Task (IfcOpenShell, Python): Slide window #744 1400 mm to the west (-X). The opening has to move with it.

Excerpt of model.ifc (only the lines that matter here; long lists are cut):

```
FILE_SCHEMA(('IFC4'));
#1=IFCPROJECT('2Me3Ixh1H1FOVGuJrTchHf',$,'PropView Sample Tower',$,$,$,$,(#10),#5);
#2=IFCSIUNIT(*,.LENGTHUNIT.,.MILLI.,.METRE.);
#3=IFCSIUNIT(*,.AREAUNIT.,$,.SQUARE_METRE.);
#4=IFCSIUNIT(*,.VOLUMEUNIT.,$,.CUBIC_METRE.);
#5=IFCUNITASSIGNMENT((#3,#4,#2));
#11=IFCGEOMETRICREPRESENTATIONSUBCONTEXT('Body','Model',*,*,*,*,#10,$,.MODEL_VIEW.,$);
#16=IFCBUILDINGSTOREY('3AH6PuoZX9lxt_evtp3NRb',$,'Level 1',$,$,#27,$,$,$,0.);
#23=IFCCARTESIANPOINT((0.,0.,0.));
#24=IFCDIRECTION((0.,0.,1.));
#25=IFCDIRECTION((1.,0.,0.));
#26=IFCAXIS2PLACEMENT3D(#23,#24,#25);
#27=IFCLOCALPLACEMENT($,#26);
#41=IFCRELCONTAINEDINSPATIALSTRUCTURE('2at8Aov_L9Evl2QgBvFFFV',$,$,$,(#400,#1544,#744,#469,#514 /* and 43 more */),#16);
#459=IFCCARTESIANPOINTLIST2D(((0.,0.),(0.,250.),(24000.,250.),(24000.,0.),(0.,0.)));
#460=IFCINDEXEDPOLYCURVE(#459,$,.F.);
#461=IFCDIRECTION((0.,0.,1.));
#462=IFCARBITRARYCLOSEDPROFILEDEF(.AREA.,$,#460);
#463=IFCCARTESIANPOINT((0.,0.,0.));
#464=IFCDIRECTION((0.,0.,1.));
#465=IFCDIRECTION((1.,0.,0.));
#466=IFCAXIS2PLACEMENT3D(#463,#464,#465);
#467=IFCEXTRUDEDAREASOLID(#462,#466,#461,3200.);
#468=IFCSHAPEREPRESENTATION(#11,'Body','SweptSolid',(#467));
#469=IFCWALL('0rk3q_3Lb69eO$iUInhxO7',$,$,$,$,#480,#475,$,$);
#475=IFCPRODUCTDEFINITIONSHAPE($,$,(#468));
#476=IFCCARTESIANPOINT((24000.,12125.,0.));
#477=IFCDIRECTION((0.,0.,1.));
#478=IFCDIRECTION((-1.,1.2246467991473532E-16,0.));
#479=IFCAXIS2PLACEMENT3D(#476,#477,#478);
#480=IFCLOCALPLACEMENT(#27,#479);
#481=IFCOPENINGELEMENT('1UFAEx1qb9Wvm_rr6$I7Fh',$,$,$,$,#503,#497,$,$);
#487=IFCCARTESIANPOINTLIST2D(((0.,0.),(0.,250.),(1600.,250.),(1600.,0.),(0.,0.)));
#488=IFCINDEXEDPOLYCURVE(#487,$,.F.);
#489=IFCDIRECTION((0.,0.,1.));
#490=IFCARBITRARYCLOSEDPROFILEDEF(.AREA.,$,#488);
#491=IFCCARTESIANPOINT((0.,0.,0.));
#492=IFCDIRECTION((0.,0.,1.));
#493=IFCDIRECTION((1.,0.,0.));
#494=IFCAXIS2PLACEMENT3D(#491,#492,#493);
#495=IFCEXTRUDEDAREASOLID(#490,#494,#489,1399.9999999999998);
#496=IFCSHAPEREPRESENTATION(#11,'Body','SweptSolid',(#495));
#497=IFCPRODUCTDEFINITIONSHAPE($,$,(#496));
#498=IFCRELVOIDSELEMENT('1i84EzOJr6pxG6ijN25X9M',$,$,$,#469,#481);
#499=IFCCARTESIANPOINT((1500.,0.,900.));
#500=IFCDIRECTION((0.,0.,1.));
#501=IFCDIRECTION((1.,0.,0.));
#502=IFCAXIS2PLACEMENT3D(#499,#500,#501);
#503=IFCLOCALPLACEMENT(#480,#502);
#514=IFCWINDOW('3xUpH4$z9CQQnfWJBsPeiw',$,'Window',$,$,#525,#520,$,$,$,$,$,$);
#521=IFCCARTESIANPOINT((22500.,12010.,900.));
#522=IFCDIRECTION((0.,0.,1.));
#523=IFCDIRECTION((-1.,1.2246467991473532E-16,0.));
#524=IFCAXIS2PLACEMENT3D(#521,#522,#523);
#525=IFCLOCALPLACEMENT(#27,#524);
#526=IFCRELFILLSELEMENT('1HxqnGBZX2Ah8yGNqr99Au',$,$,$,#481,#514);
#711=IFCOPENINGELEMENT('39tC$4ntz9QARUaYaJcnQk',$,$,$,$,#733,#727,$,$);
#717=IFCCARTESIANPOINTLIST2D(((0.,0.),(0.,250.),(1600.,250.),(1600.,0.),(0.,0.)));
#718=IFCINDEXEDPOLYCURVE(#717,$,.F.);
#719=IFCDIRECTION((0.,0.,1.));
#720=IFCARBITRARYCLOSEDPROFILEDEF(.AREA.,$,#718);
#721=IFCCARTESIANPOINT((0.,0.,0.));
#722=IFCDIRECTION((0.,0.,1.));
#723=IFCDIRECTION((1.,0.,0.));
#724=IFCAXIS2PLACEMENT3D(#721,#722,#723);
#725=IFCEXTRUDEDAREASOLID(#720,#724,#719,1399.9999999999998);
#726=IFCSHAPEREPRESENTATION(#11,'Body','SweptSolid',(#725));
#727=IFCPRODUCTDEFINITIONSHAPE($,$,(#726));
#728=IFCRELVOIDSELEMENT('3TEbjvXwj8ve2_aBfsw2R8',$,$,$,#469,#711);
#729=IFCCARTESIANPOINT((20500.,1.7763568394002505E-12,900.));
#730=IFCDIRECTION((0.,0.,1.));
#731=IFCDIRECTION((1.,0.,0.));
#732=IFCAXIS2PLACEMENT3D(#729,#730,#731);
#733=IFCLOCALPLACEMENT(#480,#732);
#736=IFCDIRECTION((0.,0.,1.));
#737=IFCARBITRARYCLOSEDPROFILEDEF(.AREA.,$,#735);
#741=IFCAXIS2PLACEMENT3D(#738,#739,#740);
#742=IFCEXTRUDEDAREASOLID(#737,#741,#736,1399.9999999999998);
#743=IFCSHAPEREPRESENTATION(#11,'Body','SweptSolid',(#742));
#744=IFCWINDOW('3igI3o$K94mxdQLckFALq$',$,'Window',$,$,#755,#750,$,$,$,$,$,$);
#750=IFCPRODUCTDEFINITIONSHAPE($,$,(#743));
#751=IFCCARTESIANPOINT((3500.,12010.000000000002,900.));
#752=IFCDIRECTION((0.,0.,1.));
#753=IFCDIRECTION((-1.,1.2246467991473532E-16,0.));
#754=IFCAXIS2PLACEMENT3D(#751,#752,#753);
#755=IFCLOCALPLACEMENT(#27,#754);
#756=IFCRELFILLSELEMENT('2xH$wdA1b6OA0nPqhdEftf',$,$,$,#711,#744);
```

```python
import ifcopenshell
import ifcopenshell.api.geometry
import ifcopenshell.util.placement

model = ifcopenshell.open("model.ifc")

window = model.by_guid("3igI3o$K94mxdQLckFALq$")
opening = window.FillsVoids[0].RelatingOpeningElement
wall = opening.VoidsElements[0].RelatingBuildingElement

wall_matrix = ifcopenshell.util.placement.get_local_placement(wall.ObjectPlacement)
shift = wall_matrix[:3, 0] * 1400.0
before = ifcopenshell.util.placement.get_local_placement(window.ObjectPlacement)[:3, 3].copy()

# The window is not placed relative to its opening, so move both.
for product in (opening, window):
    matrix = ifcopenshell.util.placement.get_local_placement(product.ObjectPlacement)
    matrix[:3, 3] += shift
    ifcopenshell.api.geometry.edit_object_placement(model, product=product, matrix=matrix, is_si=False)

after = ifcopenshell.util.placement.get_local_placement(window.ObjectPlacement)[:3, 3]
print("window moved by", (after - before).round(3) + 0.0)

model.write("model_edited.ifc")
```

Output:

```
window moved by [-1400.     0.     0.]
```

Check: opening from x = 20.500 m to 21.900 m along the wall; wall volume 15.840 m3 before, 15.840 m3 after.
